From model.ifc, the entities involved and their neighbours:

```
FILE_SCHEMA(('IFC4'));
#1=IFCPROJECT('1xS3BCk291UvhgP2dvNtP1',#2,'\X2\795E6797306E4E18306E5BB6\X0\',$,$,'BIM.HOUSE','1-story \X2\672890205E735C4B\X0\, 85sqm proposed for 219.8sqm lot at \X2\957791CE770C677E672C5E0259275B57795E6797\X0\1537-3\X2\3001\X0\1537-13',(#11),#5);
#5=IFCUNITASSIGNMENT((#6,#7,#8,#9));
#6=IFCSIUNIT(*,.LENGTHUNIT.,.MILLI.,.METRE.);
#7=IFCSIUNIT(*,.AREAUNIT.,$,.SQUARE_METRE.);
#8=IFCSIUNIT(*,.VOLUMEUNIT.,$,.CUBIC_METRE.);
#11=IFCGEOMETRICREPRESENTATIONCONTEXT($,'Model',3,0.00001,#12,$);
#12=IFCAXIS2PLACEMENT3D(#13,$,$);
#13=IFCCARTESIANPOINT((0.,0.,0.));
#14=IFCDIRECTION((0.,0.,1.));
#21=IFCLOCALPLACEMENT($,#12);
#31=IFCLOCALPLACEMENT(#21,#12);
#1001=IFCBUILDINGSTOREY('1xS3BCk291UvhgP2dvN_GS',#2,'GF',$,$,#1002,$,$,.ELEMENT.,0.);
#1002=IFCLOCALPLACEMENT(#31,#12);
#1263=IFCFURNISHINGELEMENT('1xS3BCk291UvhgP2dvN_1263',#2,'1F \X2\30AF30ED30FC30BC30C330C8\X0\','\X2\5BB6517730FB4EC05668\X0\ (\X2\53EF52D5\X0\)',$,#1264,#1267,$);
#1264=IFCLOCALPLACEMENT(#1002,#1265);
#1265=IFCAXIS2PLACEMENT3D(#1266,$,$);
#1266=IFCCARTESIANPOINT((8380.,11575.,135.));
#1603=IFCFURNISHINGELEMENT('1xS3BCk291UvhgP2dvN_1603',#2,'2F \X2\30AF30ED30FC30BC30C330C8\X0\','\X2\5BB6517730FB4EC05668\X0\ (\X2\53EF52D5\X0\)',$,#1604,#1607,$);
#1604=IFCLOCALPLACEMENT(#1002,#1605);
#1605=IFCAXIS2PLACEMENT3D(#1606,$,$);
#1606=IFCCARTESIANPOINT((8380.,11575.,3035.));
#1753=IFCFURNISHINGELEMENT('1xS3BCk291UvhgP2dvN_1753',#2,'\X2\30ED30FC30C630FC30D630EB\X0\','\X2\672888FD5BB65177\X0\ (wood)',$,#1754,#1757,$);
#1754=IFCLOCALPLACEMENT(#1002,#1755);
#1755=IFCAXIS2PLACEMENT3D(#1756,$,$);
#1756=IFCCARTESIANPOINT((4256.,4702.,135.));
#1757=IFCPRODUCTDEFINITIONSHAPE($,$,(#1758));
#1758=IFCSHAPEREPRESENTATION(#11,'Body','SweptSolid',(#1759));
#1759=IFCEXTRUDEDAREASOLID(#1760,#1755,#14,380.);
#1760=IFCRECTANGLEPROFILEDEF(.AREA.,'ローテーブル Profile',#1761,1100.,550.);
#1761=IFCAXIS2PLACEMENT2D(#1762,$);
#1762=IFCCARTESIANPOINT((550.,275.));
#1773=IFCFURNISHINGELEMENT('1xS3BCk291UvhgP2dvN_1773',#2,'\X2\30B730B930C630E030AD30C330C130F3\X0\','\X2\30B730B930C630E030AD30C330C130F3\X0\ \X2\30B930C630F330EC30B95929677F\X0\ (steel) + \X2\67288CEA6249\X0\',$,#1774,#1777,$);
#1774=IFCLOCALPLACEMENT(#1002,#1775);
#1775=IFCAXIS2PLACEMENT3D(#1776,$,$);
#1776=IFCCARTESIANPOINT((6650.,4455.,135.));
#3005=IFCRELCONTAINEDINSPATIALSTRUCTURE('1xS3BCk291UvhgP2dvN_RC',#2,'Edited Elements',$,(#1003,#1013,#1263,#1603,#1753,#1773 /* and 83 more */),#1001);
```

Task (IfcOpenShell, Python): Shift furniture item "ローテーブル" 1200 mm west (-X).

```python
import ifcopenshell
import ifcopenshell.api.geometry
import ifcopenshell.util.placement

model = ifcopenshell.open("model.ifc")

item = model.by_guid("1xS3BCk291UvhgP2dvN_1753")
matrix = ifcopenshell.util.placement.get_local_placement(item.ObjectPlacement)
matrix[0, 3] -= 1200.0
ifcopenshell.api.geometry.edit_object_placement(model, product=item, matrix=matrix, is_si=False)

print(ifcopenshell.util.placement.get_local_placement(item.ObjectPlacement).round(3) + 0.0)

model.write("model_updated.ifc")
```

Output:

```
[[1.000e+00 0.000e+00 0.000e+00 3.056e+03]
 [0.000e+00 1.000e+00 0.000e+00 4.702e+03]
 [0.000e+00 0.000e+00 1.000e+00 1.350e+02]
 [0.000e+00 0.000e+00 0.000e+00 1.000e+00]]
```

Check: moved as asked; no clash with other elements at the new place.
